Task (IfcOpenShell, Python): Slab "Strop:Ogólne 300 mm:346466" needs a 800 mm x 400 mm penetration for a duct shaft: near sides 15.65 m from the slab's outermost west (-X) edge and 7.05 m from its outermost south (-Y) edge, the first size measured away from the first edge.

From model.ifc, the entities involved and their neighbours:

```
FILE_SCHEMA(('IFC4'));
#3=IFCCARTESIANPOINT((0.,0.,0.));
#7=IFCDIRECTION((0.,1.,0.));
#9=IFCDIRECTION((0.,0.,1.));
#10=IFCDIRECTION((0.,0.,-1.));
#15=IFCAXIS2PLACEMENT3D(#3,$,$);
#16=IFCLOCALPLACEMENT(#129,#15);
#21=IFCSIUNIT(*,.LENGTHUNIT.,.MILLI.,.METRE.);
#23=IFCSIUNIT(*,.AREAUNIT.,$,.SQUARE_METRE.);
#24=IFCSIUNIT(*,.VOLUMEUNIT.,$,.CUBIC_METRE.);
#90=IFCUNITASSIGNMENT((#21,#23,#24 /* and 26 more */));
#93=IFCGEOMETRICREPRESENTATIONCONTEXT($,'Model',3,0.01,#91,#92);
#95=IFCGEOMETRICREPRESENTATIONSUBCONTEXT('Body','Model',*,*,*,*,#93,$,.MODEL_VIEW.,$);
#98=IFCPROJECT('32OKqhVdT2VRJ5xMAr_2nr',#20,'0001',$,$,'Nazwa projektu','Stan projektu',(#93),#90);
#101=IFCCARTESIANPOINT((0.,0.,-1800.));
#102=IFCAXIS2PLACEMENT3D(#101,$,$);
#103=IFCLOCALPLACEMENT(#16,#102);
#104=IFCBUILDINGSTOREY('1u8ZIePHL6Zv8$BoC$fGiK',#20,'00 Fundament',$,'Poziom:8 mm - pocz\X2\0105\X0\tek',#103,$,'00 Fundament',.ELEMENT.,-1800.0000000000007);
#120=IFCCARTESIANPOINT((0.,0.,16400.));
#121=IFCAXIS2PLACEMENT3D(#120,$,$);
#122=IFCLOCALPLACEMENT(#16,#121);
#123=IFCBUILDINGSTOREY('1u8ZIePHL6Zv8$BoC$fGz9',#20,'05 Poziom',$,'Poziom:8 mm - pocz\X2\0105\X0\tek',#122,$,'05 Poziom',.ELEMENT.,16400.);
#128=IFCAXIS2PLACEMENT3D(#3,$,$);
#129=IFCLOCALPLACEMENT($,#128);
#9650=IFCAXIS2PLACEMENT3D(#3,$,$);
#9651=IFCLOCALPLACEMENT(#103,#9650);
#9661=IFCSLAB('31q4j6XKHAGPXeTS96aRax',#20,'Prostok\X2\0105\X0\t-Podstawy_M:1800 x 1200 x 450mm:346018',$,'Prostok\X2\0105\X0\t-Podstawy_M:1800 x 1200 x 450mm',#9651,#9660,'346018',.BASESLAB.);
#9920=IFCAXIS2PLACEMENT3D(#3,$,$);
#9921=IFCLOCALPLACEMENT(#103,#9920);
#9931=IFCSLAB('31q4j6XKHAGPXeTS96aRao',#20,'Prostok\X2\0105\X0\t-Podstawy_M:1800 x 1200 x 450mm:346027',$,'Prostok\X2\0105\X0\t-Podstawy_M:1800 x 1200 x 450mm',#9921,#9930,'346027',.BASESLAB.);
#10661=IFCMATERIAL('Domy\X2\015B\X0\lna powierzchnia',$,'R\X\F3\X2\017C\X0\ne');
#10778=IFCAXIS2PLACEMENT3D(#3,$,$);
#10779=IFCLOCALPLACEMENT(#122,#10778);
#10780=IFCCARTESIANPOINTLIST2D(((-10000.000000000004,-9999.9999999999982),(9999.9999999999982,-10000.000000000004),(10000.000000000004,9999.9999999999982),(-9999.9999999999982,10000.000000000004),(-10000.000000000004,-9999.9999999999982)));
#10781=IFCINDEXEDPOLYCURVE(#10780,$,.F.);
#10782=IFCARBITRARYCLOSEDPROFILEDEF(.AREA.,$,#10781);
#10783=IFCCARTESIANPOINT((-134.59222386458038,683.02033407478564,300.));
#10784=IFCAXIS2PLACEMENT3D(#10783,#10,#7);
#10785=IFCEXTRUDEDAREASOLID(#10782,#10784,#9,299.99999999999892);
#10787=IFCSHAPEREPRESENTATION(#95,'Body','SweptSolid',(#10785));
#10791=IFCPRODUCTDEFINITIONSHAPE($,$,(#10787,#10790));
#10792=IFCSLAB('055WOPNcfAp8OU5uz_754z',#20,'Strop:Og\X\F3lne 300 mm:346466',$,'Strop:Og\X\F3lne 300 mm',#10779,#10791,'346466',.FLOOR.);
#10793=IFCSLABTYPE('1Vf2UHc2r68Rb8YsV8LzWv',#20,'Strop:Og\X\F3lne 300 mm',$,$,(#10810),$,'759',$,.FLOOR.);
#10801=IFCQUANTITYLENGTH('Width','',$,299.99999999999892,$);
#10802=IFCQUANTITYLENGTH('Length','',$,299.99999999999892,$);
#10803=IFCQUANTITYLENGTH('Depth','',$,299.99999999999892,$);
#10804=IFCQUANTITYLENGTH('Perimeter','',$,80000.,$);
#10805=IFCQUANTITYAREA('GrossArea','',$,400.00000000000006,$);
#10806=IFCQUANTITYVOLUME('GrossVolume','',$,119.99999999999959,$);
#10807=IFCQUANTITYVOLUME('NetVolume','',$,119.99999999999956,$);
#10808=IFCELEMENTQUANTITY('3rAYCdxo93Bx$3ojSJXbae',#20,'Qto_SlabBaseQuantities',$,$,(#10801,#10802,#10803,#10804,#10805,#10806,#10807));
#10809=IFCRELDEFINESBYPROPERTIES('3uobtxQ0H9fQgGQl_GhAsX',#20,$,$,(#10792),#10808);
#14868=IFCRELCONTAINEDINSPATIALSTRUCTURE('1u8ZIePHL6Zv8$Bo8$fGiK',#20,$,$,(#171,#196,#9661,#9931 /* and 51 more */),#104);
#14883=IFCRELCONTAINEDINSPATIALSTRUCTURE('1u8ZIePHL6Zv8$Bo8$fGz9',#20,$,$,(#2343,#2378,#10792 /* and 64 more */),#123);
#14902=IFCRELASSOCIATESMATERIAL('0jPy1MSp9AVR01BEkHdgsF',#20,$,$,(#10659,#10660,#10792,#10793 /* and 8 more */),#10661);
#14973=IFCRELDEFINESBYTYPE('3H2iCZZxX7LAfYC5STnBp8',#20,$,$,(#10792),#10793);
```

```python
import numpy as np
import ifcopenshell
import ifcopenshell.api.feature
import ifcopenshell.api.geometry
import ifcopenshell.api.pset
import ifcopenshell.api.root
import ifcopenshell.geom
import ifcopenshell.util.element
import ifcopenshell.util.placement
import ifcopenshell.util.representation
import ifcopenshell.util.shape
import ifcopenshell.util.unit

model = ifcopenshell.open("model.ifc")
unit_scale = ifcopenshell.util.unit.calculate_unit_scale(model)
volume_scale = ifcopenshell.util.unit.calculate_unit_scale(model, "VOLUMEUNIT")
settings = ifcopenshell.geom.settings()


def volume(element):
    """Net volume in cubic metres, openings subtracted."""
    shape = ifcopenshell.geom.create_shape(settings, element)
    return ifcopenshell.util.shape.get_volume(shape.geometry)


slab = model.by_guid("055WOPNcfAp8OU5uz_754z")
before = volume(slab)

# Extent in the slab's own axes, in metres. The edges named are its -X and -Y sides.
slab_shape = ifcopenshell.geom.create_shape(settings, slab)
vertices = ifcopenshell.util.shape.get_vertices(slab_shape.geometry)
x_min, y_min, bottom = vertices.min(axis=0)
top = vertices[:, 2].max()

opening = ifcopenshell.api.root.create_entity(model, ifc_class="IfcOpeningElement", name="Duct shaft opening", predefined_type="OPENING")
context = ifcopenshell.util.representation.get_context(model, "Model", "Body", "MODEL_VIEW")
width, depth = 0.8, 0.4
outline = [(0.0, 0.0), (width, 0.0), (width, depth), (0.0, depth), (0.0, 0.0)]
# Overshoot both faces by 50 mm so the cut is clean.
shape = ifcopenshell.api.geometry.add_slab_representation(
    model, context=context, depth=top - bottom + 0.1, polyline=outline
)
ifcopenshell.api.geometry.assign_representation(model, product=opening, representation=shape)

matrix = ifcopenshell.util.placement.get_local_placement(slab.ObjectPlacement)
matrix[:, 3] = matrix @ np.append(np.array([x_min + 15.65, y_min + 7.05, bottom - 0.05]) / unit_scale, 1.0)
ifcopenshell.api.geometry.edit_object_placement(model, product=opening, matrix=matrix, is_si=False)
ifcopenshell.api.feature.add_feature(model, feature=opening, element=slab)

after = volume(slab)

# Update the slab's stored quantities.
qto = model.by_id(ifcopenshell.util.element.get_pset(slab, "Qto_SlabBaseQuantities", should_inherit=False)["id"])
ifcopenshell.api.pset.edit_qto(model, qto=qto, properties={"NetVolume": after / volume_scale})

print(f"slab volume {before:.3f} -> {after:.3f} m3")

model.write("model-out.ifc")
```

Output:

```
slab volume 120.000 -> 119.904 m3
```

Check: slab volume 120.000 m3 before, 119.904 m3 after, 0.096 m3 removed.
